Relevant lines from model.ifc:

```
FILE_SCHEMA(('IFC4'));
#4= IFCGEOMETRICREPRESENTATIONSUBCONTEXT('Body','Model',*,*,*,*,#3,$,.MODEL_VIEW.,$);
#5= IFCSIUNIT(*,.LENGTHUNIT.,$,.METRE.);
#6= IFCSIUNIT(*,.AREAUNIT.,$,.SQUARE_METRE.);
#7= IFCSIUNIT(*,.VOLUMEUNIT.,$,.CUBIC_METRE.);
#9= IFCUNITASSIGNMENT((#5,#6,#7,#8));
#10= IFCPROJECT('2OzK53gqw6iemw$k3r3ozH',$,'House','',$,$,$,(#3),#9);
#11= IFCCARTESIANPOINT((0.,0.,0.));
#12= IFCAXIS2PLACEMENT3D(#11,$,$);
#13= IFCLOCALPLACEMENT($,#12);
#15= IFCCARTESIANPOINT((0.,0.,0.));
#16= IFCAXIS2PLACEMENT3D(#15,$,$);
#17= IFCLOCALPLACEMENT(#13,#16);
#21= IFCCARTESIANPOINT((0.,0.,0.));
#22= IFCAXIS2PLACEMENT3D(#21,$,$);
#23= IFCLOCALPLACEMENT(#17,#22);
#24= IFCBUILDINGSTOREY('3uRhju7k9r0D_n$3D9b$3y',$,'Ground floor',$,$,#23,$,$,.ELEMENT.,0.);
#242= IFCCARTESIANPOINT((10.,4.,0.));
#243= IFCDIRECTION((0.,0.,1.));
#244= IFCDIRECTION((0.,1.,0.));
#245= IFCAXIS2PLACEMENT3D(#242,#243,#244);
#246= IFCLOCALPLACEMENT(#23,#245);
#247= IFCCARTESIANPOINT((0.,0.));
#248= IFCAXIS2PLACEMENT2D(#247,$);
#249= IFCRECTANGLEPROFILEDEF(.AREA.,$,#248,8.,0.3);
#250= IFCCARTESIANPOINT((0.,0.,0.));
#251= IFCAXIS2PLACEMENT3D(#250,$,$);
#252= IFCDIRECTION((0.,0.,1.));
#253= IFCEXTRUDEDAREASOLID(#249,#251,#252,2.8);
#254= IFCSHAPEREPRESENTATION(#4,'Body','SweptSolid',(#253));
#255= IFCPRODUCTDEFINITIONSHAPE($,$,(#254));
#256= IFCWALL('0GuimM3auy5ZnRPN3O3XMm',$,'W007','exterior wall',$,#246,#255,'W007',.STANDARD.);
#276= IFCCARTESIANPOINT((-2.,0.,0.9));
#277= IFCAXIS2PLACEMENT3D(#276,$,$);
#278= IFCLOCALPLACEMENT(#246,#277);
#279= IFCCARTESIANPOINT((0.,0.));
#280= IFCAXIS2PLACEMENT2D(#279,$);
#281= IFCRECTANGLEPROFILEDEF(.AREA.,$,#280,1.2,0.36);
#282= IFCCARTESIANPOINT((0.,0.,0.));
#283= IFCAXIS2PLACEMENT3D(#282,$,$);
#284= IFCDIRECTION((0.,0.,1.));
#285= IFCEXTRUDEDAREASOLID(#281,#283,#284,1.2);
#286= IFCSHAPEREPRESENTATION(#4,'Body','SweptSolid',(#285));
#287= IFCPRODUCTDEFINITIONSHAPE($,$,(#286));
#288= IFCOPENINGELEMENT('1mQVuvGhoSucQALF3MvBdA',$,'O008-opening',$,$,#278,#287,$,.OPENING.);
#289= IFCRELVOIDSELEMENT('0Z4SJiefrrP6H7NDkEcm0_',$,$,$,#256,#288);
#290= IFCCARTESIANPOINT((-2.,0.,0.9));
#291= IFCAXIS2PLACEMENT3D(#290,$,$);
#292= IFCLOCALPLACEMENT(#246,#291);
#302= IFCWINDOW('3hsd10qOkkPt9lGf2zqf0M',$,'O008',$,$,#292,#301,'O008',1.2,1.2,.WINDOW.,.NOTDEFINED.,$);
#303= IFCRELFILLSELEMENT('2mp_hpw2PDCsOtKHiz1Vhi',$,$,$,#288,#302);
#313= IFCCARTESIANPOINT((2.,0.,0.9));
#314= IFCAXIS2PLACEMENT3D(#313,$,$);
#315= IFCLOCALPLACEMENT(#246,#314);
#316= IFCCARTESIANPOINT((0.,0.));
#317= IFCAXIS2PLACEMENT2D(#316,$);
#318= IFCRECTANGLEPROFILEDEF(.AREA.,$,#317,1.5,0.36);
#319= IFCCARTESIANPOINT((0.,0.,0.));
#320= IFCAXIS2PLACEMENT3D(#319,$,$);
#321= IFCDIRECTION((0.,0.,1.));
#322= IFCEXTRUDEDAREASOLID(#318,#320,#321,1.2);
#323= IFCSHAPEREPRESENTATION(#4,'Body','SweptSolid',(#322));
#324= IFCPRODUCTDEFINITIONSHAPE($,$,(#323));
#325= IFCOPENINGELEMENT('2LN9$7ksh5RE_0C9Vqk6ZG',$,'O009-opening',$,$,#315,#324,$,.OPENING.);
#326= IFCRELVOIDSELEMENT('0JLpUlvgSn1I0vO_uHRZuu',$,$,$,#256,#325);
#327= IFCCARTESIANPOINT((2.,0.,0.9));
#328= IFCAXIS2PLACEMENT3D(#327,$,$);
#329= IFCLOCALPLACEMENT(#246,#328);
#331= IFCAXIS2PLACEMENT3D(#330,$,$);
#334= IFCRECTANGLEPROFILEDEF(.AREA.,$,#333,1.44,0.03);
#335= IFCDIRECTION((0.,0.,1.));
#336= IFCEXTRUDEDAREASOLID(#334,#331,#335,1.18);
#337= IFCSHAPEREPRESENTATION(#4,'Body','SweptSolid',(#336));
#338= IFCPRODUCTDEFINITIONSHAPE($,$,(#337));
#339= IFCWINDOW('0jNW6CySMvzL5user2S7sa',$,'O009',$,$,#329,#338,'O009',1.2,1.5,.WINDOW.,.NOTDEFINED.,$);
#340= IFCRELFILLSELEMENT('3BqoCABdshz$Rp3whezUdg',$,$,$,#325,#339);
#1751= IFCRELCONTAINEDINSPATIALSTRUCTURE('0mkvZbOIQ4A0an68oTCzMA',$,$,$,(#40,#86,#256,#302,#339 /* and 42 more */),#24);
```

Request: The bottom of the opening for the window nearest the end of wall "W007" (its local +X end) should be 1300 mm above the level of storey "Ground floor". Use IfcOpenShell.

```python
import numpy as np
import ifcopenshell
import ifcopenshell.api.geometry
import ifcopenshell.geom
import ifcopenshell.util.element
import ifcopenshell.util.placement
import ifcopenshell.util.shape
import ifcopenshell.util.unit

model = ifcopenshell.open("model.ifc")
unit_scale = ifcopenshell.util.unit.calculate_unit_scale(model)

window = model.by_guid("0jNW6CySMvzL5user2S7sa")
opening = window.FillsVoids[0].RelatingOpeningElement
storey = ifcopenshell.util.element.get_container(window, ifc_class="IfcBuildingStorey")
level = ifcopenshell.util.placement.get_local_placement(storey.ObjectPlacement)[2, 3]

# The opening's origin need not be at the sill, so measure its lowest point.
shape = ifcopenshell.geom.create_shape(ifcopenshell.geom.settings(), opening)
bottom = ifcopenshell.util.shape.get_shape_bottom_elevation(shape, shape.geometry) / unit_scale
dz = level + 1.3 - bottom

shift = np.array([0.0, 0.0, dz])
# The window is not placed relative to its opening, so move both.
for product in (opening, window):
    matrix = ifcopenshell.util.placement.get_local_placement(product.ObjectPlacement)
    matrix[:3, 3] += shift
    ifcopenshell.api.geometry.edit_object_placement(model, product=product, matrix=matrix, is_si=False)

print(f"moved by {dz * unit_scale:+.3f} m")

model.write("model-out.ifc")
```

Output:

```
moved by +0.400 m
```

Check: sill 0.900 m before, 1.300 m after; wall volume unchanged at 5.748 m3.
